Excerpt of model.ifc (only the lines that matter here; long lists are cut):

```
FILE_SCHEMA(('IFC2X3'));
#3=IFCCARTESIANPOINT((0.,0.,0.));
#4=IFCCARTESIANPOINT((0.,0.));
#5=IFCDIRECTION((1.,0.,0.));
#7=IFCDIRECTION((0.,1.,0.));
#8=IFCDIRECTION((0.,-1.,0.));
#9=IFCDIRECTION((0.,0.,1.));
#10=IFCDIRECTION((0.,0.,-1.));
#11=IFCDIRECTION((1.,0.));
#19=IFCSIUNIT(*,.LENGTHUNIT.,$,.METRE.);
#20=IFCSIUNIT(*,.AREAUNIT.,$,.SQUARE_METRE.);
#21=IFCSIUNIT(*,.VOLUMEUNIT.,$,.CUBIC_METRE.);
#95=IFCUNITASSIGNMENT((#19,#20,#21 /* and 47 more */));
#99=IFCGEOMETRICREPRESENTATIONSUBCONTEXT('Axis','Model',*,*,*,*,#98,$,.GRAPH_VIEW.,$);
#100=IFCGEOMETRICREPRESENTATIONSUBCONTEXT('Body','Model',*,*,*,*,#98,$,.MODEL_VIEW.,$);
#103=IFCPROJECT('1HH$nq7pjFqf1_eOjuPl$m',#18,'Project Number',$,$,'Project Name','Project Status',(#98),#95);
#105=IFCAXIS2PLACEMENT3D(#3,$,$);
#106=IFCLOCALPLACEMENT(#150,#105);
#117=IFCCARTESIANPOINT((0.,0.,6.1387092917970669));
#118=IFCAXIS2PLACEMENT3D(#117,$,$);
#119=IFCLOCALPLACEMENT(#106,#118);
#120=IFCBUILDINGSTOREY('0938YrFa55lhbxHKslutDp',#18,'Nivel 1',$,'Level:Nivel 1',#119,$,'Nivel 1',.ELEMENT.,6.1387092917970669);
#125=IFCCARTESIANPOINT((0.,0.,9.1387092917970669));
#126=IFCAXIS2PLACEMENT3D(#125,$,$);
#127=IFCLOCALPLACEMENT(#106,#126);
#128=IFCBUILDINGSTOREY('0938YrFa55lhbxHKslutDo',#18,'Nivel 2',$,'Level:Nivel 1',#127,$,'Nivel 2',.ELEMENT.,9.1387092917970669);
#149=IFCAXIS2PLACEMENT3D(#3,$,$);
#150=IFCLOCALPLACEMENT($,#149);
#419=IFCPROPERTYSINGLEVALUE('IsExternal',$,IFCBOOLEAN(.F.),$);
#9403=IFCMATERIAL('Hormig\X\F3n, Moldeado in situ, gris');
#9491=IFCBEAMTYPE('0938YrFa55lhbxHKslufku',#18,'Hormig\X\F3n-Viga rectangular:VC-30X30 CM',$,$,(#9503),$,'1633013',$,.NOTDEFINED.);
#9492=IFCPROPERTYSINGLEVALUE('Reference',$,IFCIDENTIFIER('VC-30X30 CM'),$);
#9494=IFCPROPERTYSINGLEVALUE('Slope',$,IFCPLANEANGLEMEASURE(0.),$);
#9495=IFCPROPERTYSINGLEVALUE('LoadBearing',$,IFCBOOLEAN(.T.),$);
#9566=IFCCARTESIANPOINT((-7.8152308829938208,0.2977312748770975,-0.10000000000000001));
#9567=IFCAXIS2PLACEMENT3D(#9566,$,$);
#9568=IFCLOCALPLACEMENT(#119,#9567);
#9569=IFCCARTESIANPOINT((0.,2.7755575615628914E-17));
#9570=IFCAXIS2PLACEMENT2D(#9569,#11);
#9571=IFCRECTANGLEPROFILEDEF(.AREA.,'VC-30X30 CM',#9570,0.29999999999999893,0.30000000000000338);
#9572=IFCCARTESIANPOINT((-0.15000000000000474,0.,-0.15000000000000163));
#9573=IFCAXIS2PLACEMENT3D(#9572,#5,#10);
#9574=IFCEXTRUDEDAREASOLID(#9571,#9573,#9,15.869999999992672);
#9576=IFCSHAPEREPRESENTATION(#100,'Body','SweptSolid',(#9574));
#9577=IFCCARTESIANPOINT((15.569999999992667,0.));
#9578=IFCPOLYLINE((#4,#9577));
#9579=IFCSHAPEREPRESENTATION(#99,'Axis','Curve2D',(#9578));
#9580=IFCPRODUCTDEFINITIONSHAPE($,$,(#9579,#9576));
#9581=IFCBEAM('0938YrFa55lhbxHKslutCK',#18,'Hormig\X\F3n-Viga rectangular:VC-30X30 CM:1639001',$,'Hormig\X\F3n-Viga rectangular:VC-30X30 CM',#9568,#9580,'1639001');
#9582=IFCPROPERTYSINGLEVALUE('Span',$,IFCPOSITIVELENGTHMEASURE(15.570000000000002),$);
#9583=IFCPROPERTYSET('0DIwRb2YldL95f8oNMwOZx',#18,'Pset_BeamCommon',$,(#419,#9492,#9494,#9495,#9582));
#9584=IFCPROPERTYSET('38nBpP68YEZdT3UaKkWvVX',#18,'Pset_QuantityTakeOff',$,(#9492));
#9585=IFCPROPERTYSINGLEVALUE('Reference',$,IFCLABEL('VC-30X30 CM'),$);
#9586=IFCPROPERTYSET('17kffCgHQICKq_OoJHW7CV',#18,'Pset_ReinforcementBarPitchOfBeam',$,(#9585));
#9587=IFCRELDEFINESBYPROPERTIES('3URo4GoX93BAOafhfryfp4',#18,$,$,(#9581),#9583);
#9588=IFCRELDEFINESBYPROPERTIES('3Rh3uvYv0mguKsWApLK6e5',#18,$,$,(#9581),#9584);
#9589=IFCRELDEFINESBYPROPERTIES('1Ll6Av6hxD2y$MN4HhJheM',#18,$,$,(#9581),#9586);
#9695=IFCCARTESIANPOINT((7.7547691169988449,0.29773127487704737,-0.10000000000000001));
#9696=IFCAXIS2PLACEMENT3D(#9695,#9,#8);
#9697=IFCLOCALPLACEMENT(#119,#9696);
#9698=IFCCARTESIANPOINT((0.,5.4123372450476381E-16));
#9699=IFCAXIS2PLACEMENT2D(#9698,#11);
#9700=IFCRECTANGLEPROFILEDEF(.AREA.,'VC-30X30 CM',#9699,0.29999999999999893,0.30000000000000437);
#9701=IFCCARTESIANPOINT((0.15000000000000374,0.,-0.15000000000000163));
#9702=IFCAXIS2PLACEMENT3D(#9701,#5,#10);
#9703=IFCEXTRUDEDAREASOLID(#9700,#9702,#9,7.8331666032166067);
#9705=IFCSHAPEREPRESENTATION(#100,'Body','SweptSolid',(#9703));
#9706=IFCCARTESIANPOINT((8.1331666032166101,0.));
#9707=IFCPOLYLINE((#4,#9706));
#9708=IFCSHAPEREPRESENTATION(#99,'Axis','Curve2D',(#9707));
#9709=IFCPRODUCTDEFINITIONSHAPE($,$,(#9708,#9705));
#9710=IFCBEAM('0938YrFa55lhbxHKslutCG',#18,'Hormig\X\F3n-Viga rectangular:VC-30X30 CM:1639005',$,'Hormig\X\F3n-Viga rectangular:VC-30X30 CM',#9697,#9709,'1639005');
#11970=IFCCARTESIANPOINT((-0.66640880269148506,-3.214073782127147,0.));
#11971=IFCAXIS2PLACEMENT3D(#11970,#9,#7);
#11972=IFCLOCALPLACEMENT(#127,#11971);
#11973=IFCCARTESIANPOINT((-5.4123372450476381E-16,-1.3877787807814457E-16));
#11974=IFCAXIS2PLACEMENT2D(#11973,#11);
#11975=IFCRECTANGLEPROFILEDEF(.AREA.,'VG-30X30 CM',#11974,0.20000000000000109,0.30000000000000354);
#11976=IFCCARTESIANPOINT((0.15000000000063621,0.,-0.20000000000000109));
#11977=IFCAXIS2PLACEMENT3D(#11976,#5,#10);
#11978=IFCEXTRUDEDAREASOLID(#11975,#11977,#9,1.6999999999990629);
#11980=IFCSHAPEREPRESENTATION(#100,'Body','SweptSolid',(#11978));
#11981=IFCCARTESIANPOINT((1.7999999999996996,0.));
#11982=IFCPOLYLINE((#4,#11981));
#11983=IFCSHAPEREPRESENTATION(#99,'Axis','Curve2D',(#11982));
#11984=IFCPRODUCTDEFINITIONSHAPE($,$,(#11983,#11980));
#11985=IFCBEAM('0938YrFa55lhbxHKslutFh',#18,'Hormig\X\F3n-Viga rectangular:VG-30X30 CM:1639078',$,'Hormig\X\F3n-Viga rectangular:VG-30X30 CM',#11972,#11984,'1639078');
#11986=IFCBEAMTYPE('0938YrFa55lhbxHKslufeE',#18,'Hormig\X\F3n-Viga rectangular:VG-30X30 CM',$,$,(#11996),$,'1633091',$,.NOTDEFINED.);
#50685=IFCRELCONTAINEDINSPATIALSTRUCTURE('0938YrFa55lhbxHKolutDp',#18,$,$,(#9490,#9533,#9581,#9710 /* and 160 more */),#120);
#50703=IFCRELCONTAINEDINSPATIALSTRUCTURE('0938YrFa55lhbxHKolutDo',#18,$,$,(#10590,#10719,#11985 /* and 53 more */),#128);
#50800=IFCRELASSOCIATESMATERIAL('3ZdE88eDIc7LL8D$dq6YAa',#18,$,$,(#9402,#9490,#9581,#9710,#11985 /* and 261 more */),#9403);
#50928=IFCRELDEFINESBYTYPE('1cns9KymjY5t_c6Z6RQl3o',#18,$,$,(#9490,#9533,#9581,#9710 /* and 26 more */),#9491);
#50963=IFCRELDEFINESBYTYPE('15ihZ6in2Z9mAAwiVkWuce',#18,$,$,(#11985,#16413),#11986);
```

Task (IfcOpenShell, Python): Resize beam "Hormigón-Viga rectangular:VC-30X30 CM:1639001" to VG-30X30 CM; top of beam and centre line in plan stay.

```python
import ifcopenshell
import ifcopenshell.api.pset
import ifcopenshell.api.type
import ifcopenshell.util.element
import ifcopenshell.util.representation

model = ifcopenshell.open("model.ifc")

member = model.by_id(9581)
source = next(p for p in model.by_type("IfcRectangleProfileDef") if p.ProfileName == "VG-30X30 CM")

body = ifcopenshell.util.representation.get_representation(member, "Model", "Body")
solid = body.Items[0]
old_profile = solid.SweptArea

# Copy the section's sizes but keep this member's own profile position.
profile = ifcopenshell.util.element.copy(model, source)
# Profiles are centred, so shift by half the change in depth to hold the top.
shift = (old_profile.XDim - profile.XDim) / 2
x, y = old_profile.Position.Location.Coordinates
up = (-1.0, 0.0)  # upwards, in the solid's own plane
location = model.createIfcCartesianPoint((x + up[0] * shift, y + up[1] * shift))
profile.Position = model.createIfcAxis2Placement2D(location, old_profile.Position.RefDirection)
solid.SweptArea = profile
if not model.get_total_inverses(old_profile):
    ifcopenshell.util.element.remove_deep2(model, old_profile)

new_type = model.by_guid("0938YrFa55lhbxHKslufeE")
ifcopenshell.api.type.assign_type(
    model, related_objects=[member], relating_type=new_type, should_map_representations=False
)
member.Name = member.Name.replace("VC-30X30 CM", "VG-30X30 CM")
member.ObjectType = "Hormigón-Viga rectangular:VG-30X30 CM"
pset = model.by_id(ifcopenshell.util.element.get_pset(member, "Pset_BeamCommon", should_inherit=False)["id"])
ifcopenshell.api.pset.edit_pset(model, pset=pset, properties={"Reference": "VG-30X30 CM"})
pset = model.by_id(ifcopenshell.util.element.get_pset(member, "Pset_QuantityTakeOff", should_inherit=False)["id"])
ifcopenshell.api.pset.edit_pset(model, pset=pset, properties={"Reference": "VG-30X30 CM"})
pset = model.by_id(ifcopenshell.util.element.get_pset(member, "Pset_ReinforcementBarPitchOfBeam", should_inherit=False)["id"])
ifcopenshell.api.pset.edit_pset(model, pset=pset, properties={"Reference": "VG-30X30 CM"})

print(solid.SweptArea)

model.write("model_rev.ifc")
```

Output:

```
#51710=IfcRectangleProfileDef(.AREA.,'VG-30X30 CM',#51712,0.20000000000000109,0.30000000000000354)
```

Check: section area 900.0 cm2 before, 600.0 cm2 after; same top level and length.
